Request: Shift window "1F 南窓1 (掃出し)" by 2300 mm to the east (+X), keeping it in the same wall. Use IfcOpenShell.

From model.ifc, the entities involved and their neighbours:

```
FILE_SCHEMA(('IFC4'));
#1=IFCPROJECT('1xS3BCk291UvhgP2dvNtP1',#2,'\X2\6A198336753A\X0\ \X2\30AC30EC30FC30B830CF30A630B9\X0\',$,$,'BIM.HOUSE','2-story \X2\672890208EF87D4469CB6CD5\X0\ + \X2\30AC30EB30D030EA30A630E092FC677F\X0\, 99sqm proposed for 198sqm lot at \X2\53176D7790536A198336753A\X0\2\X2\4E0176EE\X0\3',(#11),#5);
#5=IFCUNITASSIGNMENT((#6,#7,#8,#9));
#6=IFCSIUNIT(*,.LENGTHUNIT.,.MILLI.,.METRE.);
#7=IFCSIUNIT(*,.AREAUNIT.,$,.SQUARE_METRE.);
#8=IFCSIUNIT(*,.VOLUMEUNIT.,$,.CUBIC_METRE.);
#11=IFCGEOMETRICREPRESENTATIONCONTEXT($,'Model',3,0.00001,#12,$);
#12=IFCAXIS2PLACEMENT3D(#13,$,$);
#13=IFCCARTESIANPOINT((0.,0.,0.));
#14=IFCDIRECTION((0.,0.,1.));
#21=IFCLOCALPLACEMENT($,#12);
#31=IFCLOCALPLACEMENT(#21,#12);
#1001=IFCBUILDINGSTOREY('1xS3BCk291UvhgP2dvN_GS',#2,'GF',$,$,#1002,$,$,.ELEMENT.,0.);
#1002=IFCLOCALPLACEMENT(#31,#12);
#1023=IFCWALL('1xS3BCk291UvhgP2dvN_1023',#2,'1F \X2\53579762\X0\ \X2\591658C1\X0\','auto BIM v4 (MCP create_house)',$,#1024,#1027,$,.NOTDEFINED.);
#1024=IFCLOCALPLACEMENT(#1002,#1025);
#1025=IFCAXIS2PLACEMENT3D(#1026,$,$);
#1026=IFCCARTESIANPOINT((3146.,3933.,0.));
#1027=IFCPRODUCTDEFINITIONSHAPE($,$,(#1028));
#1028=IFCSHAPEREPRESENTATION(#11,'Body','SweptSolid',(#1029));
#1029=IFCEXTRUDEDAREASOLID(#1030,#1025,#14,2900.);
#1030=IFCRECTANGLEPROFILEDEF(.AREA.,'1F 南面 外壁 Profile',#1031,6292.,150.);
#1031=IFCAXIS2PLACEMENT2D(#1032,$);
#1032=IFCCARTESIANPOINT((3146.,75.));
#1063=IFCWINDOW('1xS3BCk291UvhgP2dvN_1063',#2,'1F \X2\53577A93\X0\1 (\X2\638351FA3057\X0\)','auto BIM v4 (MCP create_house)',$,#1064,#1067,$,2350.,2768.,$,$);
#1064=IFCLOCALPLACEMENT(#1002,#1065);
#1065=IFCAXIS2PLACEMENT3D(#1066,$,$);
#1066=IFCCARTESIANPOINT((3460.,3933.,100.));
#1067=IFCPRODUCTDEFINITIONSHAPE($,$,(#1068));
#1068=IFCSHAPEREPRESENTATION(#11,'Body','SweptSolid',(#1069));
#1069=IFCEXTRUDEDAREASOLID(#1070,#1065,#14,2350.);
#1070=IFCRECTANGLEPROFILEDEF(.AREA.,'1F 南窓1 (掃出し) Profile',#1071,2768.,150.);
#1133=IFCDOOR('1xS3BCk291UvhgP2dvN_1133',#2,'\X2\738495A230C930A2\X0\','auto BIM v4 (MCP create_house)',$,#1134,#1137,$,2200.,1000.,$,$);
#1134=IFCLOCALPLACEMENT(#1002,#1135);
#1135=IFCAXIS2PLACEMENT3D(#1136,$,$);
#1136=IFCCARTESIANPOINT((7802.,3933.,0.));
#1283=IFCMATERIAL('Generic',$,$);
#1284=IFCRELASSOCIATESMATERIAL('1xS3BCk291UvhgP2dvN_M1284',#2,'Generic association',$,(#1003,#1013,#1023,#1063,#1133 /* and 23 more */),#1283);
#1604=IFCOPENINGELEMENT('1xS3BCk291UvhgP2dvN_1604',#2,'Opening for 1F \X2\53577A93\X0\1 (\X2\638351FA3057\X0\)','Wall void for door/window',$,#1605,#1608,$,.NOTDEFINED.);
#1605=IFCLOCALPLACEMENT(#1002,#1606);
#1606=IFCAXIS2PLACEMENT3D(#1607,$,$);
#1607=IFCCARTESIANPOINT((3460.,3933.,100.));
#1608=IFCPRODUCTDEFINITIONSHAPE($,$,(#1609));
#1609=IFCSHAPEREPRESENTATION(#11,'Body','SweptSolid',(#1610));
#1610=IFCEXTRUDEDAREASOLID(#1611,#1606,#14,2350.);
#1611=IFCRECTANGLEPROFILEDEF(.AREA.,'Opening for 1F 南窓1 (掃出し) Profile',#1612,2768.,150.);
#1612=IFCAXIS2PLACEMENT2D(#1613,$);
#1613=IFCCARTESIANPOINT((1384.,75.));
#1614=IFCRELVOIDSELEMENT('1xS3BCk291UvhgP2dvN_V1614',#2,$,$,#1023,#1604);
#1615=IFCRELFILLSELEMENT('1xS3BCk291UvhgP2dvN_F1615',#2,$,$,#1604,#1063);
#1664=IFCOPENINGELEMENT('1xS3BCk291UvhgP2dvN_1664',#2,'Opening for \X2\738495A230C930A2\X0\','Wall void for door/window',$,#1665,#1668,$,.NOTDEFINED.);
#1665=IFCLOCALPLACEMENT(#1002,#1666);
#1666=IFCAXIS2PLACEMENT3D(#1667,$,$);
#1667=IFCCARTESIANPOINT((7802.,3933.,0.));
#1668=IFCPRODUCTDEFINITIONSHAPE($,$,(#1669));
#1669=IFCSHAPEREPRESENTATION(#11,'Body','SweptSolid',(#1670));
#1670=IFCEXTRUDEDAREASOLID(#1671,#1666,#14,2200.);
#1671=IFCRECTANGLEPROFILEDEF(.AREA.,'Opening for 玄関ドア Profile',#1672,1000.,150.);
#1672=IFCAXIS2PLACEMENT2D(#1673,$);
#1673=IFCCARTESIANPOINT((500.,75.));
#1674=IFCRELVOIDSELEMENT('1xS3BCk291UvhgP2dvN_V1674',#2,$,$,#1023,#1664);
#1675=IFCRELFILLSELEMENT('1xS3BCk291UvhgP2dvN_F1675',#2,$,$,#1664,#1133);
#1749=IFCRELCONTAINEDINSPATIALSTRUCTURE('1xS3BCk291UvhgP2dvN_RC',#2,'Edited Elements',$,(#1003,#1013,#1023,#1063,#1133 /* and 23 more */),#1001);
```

```python
import ifcopenshell
import ifcopenshell.api.geometry
import ifcopenshell.util.placement
import ifcopenshell.util.unit

model = ifcopenshell.open("model.ifc")
unit_scale = ifcopenshell.util.unit.calculate_unit_scale(model)

window = model.by_guid("1xS3BCk291UvhgP2dvN_1063")
opening = window.FillsVoids[0].RelatingOpeningElement
wall = opening.VoidsElements[0].RelatingBuildingElement

wall_matrix = ifcopenshell.util.placement.get_local_placement(wall.ObjectPlacement)
shift = wall_matrix[:3, 0] * 2.3 / unit_scale
before = ifcopenshell.util.placement.get_local_placement(window.ObjectPlacement)[:3, 3].copy()

# The window is not placed relative to its opening, so move both.
for product in (opening, window):
    matrix = ifcopenshell.util.placement.get_local_placement(product.ObjectPlacement)
    matrix[:3, 3] += shift
    ifcopenshell.api.geometry.edit_object_placement(model, product=product, matrix=matrix, is_si=False)

after = ifcopenshell.util.placement.get_local_placement(window.ObjectPlacement)[:3, 3]
print("window moved by", (after - before).round(3) + 0.0)

model.write("model-out.ifc")
```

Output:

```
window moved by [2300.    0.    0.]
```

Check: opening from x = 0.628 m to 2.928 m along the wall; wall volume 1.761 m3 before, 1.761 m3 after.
